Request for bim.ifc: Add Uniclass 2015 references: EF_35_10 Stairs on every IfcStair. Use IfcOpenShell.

First a look at what the model holds.

```python
import ifcopenshell

model = ifcopenshell.open("bim.ifc")
print(model.schema)
print("classifications:", [c.Name for c in model.by_type("IfcClassification")])
for ifc_class in ("IfcDoor", "IfcRoof", "IfcStair", "IfcWall", "IfcWindow"):
    print(ifc_class, len(model.by_type(ifc_class)))
```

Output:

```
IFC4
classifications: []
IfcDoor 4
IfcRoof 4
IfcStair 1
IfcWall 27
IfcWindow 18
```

```python
import ifcopenshell
import ifcopenshell.api.classification

model = ifcopenshell.open("bim.ifc")

system = ifcopenshell.api.classification.add_classification(model, classification="Uniclass 2015")

codes = {
    "IfcStair": ("EF_35_10", "Stairs"),
}
for ifc_class, (code, name) in codes.items():
    products = model.by_type(ifc_class)
    ifcopenshell.api.classification.add_reference(
        model, products=products, classification=system, identification=code, name=name
    )
    print(code, len(products))

model.write("bim_v2.ifc")
```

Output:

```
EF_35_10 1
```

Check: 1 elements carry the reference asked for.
